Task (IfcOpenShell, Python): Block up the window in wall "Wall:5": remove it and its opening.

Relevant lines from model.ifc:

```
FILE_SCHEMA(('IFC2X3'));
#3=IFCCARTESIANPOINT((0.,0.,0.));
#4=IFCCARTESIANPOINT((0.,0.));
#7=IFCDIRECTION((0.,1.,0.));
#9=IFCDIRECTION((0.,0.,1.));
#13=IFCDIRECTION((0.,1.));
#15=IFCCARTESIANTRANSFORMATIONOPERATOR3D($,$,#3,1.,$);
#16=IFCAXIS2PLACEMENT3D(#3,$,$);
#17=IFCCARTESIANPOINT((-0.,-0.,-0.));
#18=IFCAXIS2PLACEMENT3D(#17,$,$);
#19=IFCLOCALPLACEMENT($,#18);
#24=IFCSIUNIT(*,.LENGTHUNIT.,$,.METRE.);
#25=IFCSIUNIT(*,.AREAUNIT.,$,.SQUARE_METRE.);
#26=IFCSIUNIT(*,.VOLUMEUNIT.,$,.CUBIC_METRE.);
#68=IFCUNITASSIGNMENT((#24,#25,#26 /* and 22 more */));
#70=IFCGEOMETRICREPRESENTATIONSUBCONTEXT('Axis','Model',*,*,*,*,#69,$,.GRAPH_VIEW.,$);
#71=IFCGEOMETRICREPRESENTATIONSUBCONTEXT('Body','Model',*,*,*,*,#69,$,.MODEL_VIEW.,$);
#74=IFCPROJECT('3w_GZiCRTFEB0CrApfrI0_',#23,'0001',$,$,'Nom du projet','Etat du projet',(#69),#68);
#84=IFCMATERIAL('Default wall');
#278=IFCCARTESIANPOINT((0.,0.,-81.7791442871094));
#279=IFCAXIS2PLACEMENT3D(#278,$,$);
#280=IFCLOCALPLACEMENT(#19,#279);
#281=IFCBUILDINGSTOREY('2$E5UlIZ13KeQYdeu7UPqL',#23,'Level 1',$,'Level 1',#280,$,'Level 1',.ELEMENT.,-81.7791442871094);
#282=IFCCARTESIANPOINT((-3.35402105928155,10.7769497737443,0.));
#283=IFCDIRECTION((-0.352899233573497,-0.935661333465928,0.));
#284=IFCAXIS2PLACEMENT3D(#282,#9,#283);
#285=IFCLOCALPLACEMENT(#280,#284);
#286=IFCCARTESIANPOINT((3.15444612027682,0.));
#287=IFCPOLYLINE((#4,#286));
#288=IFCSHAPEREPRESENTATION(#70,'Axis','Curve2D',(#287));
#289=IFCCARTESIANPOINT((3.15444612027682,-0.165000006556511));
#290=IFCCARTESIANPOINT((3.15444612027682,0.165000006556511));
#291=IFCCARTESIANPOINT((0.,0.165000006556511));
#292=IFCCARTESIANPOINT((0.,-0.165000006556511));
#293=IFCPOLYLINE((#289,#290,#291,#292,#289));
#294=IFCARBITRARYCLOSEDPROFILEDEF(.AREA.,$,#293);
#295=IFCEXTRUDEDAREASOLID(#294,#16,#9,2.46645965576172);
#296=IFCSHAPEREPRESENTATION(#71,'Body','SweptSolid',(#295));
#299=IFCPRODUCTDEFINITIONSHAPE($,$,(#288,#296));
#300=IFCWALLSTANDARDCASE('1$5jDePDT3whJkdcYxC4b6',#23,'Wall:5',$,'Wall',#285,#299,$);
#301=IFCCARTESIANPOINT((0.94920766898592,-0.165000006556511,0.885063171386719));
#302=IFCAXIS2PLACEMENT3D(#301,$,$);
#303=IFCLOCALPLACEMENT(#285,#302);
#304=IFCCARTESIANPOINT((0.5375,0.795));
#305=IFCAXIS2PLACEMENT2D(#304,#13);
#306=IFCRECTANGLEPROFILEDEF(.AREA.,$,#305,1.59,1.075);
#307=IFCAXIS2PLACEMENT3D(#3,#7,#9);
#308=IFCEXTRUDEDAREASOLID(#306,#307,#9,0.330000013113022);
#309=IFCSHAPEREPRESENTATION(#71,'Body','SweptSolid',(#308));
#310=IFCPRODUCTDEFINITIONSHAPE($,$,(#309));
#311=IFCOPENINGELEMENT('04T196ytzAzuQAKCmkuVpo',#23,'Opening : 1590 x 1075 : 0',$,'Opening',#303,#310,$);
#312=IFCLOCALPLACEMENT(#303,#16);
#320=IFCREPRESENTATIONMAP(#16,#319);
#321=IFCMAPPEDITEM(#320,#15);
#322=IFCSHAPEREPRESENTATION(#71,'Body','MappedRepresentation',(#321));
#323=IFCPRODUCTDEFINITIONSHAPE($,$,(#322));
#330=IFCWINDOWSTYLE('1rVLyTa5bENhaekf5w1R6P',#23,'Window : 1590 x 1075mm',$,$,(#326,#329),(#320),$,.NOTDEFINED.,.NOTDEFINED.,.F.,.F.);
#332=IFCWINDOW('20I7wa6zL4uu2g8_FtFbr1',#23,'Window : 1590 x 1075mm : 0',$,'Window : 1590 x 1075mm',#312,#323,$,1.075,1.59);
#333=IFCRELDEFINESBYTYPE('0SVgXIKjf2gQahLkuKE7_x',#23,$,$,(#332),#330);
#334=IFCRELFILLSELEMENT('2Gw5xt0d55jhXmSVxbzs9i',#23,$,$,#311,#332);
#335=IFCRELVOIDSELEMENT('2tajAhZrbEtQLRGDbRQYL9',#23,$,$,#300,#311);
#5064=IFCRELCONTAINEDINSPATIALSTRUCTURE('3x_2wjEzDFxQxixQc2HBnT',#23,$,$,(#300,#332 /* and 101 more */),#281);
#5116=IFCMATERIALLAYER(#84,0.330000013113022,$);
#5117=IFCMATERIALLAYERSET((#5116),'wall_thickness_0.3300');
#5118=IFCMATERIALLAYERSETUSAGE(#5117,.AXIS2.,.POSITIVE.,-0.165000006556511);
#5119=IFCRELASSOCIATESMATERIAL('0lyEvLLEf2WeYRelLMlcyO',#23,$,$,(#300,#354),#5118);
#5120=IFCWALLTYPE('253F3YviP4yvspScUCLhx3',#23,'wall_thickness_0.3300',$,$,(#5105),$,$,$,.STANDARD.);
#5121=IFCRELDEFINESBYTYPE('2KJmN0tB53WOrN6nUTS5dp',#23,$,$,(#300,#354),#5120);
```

```python
import ifcopenshell
import ifcopenshell.api.feature
import ifcopenshell.api.root
import ifcopenshell.geom
import ifcopenshell.util.shape

model = ifcopenshell.open("model.ifc")
settings = ifcopenshell.geom.settings()


def volume(element):
    """Net volume in cubic metres, openings subtracted."""
    shape = ifcopenshell.geom.create_shape(settings, element)
    return ifcopenshell.util.shape.get_volume(shape.geometry)


window = model.by_guid("20I7wa6zL4uu2g8_FtFbr1")
opening = window.FillsVoids[0].RelatingOpeningElement
wall = opening.VoidsElements[0].RelatingBuildingElement
before = volume(wall)

ifcopenshell.api.root.remove_product(model, product=window)
ifcopenshell.api.feature.remove_feature(model, feature=opening)

after = volume(wall)

print(f"wall volume {before:.3f} -> {after:.3f} m3")

model.write("model_updated.ifc")
```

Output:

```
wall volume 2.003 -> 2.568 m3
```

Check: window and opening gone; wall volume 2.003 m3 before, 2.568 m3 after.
